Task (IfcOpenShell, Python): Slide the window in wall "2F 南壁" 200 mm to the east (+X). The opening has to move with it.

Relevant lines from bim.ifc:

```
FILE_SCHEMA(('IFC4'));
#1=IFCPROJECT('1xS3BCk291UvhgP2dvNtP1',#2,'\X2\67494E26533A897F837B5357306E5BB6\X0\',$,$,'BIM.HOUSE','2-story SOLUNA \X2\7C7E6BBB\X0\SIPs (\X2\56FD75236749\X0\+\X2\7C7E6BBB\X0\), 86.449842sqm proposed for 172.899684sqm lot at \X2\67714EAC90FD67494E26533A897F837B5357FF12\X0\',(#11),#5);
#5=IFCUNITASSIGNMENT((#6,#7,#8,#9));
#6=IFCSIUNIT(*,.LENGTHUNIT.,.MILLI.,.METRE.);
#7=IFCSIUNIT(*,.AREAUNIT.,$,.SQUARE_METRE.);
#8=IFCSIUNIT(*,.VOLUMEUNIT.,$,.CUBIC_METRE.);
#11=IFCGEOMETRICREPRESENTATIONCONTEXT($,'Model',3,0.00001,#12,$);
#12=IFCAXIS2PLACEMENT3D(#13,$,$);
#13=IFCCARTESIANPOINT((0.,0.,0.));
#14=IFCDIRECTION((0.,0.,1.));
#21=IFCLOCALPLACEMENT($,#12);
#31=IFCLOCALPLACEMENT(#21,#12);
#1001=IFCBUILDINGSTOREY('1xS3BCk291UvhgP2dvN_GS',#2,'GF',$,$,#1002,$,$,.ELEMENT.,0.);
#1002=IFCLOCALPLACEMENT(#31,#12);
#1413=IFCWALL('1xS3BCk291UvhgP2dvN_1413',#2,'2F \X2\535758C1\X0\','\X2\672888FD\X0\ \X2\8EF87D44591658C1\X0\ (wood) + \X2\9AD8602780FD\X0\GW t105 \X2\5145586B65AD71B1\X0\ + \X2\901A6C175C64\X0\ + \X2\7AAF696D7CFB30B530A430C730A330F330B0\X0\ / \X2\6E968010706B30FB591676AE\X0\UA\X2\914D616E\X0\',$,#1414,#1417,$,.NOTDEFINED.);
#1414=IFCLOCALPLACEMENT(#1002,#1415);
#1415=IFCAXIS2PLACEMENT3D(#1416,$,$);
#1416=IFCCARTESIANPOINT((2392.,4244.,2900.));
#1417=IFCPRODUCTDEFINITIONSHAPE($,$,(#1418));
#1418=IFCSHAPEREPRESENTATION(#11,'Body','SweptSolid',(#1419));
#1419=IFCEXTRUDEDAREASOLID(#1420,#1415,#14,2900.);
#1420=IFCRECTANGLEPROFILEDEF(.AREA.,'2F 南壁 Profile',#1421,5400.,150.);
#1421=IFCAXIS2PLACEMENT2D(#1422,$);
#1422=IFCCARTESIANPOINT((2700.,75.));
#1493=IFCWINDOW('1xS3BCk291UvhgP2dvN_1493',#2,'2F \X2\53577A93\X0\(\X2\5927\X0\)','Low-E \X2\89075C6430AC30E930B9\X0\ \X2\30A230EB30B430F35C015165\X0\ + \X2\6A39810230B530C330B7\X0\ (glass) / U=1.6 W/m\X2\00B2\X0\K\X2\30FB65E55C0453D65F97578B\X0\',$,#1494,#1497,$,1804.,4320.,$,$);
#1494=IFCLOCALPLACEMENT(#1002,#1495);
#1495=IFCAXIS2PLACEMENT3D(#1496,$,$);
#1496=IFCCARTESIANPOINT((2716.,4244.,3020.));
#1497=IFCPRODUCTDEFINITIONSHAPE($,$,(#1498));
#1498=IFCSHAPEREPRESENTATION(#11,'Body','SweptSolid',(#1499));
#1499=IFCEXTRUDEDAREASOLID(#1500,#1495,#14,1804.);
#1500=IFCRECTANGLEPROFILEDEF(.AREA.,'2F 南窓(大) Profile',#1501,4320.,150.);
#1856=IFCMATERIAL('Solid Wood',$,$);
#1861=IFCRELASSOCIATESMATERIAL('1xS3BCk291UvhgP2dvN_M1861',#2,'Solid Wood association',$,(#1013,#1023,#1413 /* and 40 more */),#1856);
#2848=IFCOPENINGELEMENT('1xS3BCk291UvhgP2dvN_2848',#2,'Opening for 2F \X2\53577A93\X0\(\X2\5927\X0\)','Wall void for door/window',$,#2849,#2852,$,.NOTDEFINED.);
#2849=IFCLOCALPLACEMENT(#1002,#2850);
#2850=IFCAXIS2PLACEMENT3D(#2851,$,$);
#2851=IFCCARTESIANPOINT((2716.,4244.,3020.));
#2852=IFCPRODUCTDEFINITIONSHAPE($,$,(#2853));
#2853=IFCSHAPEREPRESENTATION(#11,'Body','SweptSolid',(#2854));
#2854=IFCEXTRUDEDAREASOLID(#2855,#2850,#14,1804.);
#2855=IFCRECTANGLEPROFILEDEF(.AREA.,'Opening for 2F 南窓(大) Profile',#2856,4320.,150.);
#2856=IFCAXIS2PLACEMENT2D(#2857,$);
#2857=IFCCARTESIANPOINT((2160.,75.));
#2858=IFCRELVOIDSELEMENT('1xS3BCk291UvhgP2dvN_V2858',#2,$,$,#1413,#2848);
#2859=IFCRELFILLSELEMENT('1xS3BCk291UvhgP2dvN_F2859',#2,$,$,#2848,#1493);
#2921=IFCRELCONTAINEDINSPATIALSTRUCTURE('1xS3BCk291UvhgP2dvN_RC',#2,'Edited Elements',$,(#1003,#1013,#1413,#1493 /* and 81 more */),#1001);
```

```python
import ifcopenshell
import ifcopenshell.api.geometry
import ifcopenshell.util.placement

model = ifcopenshell.open("bim.ifc")

window = model.by_guid("1xS3BCk291UvhgP2dvN_1493")
opening = window.FillsVoids[0].RelatingOpeningElement
wall = opening.VoidsElements[0].RelatingBuildingElement

wall_matrix = ifcopenshell.util.placement.get_local_placement(wall.ObjectPlacement)
shift = wall_matrix[:3, 0] * 200.0
before = ifcopenshell.util.placement.get_local_placement(window.ObjectPlacement)[:3, 3].copy()

# The window is not placed relative to its opening, so move both.
for product in (opening, window):
    matrix = ifcopenshell.util.placement.get_local_placement(product.ObjectPlacement)
    matrix[:3, 3] += shift
    ifcopenshell.api.geometry.edit_object_placement(model, product=product, matrix=matrix, is_si=False)

after = ifcopenshell.util.placement.get_local_placement(window.ObjectPlacement)[:3, 3]
print("window moved by", (after - before).round(3) + 0.0)

model.write("bim_rev.ifc")
```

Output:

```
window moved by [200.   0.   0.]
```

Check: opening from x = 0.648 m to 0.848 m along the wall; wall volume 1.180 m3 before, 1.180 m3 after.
